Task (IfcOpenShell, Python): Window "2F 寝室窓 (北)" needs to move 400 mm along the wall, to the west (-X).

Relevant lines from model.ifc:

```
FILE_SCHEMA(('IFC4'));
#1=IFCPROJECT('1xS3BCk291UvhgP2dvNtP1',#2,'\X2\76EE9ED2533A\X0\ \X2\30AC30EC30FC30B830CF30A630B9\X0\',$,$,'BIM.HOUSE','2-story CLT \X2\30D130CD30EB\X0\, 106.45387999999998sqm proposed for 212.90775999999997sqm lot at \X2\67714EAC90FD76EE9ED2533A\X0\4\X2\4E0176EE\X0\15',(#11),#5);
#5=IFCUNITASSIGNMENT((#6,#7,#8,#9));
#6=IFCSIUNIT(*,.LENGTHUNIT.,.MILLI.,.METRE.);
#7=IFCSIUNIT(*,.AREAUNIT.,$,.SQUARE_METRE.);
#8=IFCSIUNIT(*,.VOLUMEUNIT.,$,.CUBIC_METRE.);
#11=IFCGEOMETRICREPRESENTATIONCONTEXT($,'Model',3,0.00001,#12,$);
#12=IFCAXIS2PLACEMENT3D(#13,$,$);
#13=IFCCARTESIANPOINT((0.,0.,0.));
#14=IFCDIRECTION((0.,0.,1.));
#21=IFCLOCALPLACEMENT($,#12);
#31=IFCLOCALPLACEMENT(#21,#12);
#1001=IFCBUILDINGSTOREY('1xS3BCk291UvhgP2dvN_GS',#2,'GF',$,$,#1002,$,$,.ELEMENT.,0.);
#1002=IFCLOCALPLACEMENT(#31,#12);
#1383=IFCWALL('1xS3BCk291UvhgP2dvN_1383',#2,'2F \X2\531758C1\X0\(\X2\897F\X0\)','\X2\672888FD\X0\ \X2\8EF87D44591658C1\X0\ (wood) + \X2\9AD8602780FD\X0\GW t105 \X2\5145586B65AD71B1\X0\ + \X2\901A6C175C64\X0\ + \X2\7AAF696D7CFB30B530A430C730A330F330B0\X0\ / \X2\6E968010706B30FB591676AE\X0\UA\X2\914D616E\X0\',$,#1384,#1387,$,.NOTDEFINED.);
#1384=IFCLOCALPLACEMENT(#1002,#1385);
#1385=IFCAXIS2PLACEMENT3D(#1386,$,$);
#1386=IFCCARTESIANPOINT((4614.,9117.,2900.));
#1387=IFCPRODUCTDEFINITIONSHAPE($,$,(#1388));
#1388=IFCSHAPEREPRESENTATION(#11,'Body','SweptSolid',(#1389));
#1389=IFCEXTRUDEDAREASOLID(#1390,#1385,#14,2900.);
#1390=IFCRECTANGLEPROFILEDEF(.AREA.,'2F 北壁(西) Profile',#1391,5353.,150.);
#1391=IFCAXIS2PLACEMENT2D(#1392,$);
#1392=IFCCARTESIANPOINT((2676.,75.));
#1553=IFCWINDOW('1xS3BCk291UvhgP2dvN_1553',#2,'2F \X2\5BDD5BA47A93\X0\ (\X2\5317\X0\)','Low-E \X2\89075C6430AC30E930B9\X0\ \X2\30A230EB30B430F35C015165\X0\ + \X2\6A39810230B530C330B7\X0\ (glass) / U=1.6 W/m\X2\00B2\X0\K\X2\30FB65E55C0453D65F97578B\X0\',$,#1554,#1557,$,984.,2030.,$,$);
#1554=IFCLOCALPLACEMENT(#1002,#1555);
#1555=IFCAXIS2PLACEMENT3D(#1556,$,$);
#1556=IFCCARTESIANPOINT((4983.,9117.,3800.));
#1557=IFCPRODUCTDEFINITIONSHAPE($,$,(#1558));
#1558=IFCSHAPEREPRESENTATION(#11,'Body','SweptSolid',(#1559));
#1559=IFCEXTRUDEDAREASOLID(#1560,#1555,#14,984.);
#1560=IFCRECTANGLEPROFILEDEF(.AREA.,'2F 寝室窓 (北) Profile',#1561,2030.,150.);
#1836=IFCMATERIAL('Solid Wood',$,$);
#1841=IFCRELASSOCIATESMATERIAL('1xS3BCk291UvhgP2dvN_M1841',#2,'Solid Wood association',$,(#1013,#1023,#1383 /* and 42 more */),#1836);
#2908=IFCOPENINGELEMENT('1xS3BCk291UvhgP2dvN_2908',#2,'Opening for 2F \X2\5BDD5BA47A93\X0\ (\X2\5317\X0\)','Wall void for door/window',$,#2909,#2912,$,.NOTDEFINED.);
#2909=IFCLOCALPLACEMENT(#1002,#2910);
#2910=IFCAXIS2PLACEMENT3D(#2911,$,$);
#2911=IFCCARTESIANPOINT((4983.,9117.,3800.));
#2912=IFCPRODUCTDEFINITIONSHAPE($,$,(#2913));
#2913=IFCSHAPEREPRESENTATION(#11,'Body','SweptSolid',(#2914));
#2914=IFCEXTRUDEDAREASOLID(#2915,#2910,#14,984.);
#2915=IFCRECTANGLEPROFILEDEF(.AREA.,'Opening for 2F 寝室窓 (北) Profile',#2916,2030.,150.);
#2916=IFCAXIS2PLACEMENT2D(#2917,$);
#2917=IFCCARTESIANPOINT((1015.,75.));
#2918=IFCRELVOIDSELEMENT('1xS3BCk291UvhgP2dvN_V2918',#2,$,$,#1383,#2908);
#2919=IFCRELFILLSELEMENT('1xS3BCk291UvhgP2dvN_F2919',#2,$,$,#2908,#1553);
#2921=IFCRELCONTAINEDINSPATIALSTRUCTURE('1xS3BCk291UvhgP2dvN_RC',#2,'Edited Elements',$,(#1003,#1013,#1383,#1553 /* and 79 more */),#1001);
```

```python
import ifcopenshell
import ifcopenshell.api.geometry
import ifcopenshell.util.placement

model = ifcopenshell.open("model.ifc")

window = model.by_guid("1xS3BCk291UvhgP2dvN_1553")
opening = window.FillsVoids[0].RelatingOpeningElement
wall = opening.VoidsElements[0].RelatingBuildingElement

wall_matrix = ifcopenshell.util.placement.get_local_placement(wall.ObjectPlacement)
shift = wall_matrix[:3, 0] * -400.0
before = ifcopenshell.util.placement.get_local_placement(window.ObjectPlacement)[:3, 3].copy()

# The window is not placed relative to its opening, so move both.
for product in (opening, window):
    matrix = ifcopenshell.util.placement.get_local_placement(product.ObjectPlacement)
    matrix[:3, 3] += shift
    ifcopenshell.api.geometry.edit_object_placement(model, product=product, matrix=matrix, is_si=False)

after = ifcopenshell.util.placement.get_local_placement(window.ObjectPlacement)[:3, 3]
print("window moved by", (after - before).round(3) + 0.0)

model.write("model_v2.ifc")
```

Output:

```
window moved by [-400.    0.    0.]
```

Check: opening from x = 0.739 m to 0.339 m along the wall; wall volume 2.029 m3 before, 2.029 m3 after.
